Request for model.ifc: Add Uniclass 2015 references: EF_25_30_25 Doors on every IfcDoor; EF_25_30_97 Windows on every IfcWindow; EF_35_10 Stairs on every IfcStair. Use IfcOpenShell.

First a look at what the model holds.

```python
import ifcopenshell

model = ifcopenshell.open("model.ifc")
print(model.schema)
print("classifications:", [c.Name for c in model.by_type("IfcClassification")])
for ifc_class in ("IfcDoor", "IfcRoof", "IfcStair", "IfcWall", "IfcWindow"):
    print(ifc_class, len(model.by_type(ifc_class)))
```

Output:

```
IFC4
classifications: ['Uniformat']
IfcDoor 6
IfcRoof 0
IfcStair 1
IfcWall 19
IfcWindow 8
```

```python
import ifcopenshell
import ifcopenshell.api.classification

model = ifcopenshell.open("model.ifc")

system = ifcopenshell.api.classification.add_classification(model, classification="Uniclass 2015")

codes = {
    "IfcDoor": ("EF_25_30_25", "Doors"),
    "IfcWindow": ("EF_25_30_97", "Windows"),
    "IfcStair": ("EF_35_10", "Stairs"),
}
for ifc_class, (code, name) in codes.items():
    products = model.by_type(ifc_class)
    ifcopenshell.api.classification.add_reference(
        model, products=products, classification=system, identification=code, name=name
    )
    print(code, len(products))

model.write("model_updated.ifc")
```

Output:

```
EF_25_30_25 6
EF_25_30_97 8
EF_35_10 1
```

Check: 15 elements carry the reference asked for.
